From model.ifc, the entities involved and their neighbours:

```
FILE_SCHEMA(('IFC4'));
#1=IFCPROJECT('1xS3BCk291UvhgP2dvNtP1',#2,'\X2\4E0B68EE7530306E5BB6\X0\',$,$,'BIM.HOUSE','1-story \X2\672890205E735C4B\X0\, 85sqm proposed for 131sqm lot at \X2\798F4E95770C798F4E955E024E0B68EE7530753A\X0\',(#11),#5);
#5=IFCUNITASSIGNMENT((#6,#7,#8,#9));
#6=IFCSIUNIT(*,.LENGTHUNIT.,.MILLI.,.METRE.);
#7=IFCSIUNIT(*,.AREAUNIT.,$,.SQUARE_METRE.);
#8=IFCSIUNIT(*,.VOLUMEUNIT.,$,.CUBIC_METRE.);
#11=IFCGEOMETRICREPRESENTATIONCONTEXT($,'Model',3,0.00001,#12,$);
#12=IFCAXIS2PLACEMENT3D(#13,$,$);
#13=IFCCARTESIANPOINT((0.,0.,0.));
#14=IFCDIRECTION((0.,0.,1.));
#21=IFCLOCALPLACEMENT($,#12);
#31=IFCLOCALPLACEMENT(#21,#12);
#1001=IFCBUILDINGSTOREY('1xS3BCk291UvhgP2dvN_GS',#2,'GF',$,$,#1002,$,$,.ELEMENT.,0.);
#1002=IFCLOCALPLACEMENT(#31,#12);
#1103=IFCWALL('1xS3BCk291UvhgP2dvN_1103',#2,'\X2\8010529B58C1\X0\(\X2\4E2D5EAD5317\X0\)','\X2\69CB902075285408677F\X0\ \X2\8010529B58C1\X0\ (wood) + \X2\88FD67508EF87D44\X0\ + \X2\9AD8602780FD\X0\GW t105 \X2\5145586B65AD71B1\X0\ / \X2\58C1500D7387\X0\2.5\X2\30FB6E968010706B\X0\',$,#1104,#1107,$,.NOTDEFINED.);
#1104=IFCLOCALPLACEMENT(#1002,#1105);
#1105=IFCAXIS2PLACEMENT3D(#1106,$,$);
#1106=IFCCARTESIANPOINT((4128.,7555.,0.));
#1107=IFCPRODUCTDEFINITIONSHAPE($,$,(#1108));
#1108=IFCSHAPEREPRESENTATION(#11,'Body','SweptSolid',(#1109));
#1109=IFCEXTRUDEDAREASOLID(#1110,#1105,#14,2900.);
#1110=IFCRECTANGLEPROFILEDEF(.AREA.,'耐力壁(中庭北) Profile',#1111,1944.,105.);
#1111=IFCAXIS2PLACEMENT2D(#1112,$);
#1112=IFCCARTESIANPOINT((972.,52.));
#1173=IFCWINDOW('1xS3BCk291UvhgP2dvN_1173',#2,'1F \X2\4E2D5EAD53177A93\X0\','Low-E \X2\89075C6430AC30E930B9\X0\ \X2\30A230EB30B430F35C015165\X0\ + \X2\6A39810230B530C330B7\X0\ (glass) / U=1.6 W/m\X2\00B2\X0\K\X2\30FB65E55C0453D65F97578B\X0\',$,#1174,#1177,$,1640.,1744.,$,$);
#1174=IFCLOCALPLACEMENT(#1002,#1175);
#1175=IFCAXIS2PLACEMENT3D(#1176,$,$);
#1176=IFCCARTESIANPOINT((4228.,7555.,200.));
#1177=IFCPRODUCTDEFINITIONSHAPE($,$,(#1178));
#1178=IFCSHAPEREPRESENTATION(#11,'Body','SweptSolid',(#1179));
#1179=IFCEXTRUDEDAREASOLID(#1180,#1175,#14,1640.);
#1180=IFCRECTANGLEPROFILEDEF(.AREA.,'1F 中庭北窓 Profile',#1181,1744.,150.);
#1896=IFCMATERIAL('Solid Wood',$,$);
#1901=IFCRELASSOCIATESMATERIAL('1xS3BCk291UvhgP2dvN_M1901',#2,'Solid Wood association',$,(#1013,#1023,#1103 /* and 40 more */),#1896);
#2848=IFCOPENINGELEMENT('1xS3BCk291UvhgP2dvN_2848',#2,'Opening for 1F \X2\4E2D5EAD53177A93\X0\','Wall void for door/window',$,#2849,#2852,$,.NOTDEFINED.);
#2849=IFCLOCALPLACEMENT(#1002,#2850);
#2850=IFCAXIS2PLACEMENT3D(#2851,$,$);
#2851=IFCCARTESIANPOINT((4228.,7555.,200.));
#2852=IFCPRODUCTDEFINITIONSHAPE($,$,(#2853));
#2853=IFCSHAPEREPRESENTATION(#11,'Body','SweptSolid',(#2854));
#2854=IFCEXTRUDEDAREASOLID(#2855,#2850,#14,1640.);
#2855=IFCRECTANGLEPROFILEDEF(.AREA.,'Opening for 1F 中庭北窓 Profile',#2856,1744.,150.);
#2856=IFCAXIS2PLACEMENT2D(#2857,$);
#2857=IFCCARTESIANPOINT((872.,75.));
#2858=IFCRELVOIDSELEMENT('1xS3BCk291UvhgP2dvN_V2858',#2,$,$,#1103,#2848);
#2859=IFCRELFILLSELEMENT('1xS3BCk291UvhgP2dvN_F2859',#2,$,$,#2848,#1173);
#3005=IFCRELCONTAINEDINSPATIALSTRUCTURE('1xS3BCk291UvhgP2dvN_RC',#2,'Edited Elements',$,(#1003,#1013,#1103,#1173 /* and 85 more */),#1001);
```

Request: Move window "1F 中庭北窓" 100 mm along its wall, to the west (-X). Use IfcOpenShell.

```python
import ifcopenshell
import ifcopenshell.api.geometry
import ifcopenshell.util.placement

model = ifcopenshell.open("model.ifc")

window = model.by_guid("1xS3BCk291UvhgP2dvN_1173")
opening = window.FillsVoids[0].RelatingOpeningElement
wall = opening.VoidsElements[0].RelatingBuildingElement

wall_matrix = ifcopenshell.util.placement.get_local_placement(wall.ObjectPlacement)
shift = wall_matrix[:3, 0] * -100.0
before = ifcopenshell.util.placement.get_local_placement(window.ObjectPlacement)[:3, 3].copy()

# The window is not placed relative to its opening, so move both.
for product in (opening, window):
    matrix = ifcopenshell.util.placement.get_local_placement(product.ObjectPlacement)
    matrix[:3, 3] += shift
    ifcopenshell.api.geometry.edit_object_placement(model, product=product, matrix=matrix, is_si=False)

after = ifcopenshell.util.placement.get_local_placement(window.ObjectPlacement)[:3, 3]
print("window moved by", (after - before).round(3) + 0.0)

model.write("model_updated.ifc")
```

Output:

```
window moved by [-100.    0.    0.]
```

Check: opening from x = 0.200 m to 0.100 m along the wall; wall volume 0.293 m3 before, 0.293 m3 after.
